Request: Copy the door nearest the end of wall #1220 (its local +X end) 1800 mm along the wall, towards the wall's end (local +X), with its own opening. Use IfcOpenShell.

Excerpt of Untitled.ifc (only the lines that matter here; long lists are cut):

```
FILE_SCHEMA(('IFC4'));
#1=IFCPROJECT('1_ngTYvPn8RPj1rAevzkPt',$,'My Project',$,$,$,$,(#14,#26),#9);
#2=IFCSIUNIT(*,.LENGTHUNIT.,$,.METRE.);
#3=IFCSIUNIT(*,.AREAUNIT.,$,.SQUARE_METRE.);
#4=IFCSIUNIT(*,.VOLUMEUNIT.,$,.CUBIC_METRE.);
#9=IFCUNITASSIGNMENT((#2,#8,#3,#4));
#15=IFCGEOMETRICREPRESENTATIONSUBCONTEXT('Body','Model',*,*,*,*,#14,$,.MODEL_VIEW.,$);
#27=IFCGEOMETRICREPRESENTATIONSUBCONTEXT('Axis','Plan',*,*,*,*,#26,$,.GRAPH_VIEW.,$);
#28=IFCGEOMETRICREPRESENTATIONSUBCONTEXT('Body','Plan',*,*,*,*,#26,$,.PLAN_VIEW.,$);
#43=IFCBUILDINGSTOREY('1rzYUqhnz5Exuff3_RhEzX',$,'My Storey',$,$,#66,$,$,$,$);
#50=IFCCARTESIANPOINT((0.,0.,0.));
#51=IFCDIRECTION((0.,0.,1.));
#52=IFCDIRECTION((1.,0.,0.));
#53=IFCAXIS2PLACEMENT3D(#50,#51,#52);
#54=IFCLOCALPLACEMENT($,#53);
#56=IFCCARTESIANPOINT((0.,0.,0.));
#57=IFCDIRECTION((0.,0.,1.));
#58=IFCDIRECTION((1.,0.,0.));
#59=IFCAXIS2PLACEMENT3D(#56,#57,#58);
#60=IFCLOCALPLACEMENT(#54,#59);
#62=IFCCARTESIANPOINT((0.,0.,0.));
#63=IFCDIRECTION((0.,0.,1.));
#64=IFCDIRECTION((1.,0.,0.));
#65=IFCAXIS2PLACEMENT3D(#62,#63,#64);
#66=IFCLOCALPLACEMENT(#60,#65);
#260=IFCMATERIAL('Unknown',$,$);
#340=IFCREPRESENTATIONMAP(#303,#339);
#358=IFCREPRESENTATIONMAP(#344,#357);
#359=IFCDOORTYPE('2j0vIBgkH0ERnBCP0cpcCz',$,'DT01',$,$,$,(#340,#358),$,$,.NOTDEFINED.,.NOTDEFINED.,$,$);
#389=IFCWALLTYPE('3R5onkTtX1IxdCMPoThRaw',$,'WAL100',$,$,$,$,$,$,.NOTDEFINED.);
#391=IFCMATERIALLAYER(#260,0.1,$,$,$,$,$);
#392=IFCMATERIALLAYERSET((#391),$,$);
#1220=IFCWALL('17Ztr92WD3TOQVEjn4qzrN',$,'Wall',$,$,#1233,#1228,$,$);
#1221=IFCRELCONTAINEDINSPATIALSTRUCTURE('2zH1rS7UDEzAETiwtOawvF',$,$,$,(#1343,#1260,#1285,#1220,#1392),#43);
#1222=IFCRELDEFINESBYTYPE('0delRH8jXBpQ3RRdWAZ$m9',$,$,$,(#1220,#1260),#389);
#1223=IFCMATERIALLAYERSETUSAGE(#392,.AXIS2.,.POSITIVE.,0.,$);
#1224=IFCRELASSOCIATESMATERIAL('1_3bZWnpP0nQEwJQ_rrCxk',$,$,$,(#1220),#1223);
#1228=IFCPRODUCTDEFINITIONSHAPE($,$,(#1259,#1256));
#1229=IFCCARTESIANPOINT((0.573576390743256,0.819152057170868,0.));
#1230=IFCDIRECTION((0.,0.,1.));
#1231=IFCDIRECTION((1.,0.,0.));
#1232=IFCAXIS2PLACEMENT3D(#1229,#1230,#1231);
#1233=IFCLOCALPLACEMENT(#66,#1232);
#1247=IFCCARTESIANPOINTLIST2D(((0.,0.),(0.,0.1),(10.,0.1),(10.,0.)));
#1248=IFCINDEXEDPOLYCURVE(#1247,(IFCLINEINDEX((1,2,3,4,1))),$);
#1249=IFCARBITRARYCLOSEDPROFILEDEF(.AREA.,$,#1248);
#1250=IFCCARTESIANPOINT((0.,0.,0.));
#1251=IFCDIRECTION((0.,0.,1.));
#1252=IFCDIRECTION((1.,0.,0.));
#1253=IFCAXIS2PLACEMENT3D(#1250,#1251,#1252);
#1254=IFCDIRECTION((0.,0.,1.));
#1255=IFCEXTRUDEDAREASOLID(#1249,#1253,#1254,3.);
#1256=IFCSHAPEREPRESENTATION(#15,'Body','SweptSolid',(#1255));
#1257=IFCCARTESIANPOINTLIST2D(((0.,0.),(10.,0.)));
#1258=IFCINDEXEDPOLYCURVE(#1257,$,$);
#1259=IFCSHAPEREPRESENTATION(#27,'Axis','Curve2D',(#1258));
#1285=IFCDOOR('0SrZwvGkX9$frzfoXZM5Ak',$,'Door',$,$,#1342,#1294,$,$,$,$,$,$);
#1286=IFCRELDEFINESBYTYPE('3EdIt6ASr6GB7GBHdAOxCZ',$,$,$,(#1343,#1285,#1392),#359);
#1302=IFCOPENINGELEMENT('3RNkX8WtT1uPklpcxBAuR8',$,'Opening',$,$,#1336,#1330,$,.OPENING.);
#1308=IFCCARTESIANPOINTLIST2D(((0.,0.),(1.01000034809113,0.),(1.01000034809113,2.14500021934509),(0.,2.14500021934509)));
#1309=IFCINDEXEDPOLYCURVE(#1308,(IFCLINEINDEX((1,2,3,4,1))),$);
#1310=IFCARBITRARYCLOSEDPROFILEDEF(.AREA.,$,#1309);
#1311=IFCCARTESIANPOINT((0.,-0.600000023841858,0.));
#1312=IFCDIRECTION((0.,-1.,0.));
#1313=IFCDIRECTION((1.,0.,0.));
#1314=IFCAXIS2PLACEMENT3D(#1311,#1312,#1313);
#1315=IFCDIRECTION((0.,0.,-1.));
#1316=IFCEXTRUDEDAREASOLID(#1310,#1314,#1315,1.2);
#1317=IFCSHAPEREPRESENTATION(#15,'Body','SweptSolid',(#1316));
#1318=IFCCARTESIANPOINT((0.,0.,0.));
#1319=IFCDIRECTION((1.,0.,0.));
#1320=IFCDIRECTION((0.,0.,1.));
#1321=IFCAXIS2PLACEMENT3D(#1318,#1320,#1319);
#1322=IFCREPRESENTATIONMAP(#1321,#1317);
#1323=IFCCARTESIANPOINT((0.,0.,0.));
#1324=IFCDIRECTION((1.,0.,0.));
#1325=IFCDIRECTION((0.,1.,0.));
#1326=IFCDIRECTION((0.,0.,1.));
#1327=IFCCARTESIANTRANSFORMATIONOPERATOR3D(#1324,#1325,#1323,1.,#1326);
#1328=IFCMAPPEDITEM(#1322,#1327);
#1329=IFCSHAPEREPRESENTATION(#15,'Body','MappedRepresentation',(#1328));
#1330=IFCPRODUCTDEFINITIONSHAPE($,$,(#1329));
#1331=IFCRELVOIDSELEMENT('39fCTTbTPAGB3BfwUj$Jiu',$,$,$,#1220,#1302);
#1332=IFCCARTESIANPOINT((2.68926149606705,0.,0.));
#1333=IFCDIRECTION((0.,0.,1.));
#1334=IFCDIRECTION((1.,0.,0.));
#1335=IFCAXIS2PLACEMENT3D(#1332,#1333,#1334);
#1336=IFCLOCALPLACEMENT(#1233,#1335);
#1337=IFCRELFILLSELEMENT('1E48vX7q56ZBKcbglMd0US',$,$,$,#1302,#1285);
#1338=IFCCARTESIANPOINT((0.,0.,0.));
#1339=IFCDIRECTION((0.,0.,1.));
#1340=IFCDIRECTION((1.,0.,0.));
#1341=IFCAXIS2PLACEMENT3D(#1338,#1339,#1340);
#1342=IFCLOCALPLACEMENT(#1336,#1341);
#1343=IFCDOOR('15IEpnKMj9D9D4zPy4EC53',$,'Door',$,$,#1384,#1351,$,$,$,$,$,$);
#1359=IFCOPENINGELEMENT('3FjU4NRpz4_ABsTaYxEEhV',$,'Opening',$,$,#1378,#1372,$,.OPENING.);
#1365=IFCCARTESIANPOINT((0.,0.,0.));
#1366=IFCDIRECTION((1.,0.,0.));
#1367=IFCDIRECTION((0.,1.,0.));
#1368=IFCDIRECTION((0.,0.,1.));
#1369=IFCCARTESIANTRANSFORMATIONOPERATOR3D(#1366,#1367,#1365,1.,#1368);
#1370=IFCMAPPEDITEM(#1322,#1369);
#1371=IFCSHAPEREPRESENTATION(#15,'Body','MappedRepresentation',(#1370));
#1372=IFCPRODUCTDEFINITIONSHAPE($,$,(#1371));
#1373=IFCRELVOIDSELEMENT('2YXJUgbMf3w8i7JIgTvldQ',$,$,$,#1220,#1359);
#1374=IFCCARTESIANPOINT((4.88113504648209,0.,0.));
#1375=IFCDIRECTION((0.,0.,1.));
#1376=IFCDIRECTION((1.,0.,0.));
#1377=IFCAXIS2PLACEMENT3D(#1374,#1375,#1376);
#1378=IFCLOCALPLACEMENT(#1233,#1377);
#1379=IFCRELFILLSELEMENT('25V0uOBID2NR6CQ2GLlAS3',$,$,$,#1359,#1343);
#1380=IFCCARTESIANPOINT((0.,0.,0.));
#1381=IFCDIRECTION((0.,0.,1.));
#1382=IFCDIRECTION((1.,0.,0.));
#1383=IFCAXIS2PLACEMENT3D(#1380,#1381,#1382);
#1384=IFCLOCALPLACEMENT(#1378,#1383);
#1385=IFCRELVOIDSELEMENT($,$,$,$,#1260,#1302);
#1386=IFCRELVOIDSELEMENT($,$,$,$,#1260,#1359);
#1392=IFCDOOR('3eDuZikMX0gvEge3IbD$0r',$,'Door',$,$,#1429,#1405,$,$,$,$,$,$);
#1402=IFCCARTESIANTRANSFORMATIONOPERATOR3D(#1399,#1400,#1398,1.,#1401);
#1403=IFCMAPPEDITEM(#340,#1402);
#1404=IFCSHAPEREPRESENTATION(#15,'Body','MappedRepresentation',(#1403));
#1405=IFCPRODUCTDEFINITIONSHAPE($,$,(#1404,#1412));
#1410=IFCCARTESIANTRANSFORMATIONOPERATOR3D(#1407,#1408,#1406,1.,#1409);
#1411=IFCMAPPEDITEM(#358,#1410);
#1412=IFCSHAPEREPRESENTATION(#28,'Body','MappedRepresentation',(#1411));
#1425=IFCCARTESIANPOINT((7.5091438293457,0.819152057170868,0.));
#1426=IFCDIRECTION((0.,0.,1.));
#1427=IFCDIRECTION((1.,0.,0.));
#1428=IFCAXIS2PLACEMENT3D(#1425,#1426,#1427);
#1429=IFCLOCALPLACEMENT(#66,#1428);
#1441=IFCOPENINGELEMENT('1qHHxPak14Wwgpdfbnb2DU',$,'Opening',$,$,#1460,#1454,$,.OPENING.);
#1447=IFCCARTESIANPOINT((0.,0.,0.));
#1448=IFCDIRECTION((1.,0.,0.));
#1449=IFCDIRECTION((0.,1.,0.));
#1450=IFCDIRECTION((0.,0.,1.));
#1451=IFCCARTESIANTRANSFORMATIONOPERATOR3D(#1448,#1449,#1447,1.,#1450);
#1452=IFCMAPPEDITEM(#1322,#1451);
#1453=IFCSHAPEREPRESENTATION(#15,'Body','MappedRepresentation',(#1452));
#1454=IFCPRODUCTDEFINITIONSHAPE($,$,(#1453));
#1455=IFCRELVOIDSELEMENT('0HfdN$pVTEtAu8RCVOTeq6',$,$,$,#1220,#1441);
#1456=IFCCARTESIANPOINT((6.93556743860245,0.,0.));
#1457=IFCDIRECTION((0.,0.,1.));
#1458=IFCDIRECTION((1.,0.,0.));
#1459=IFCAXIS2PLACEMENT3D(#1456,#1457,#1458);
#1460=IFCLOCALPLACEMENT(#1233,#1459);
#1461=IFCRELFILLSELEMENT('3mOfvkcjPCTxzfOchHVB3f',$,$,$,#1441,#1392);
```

```python
import ifcopenshell
import ifcopenshell.api.feature
import ifcopenshell.api.geometry
import ifcopenshell.api.root
import ifcopenshell.geom
import ifcopenshell.util.element
import ifcopenshell.util.placement
import ifcopenshell.util.shape

model = ifcopenshell.open("Untitled.ifc")
settings = ifcopenshell.geom.settings()


def volume(element):
    """Net volume in cubic metres, openings subtracted."""
    shape = ifcopenshell.geom.create_shape(settings, element)
    return ifcopenshell.util.shape.get_volume(shape.geometry)


door = model.by_guid("3eDuZikMX0gvEge3IbD$0r")
opening = door.FillsVoids[0].RelatingOpeningElement
wall = opening.VoidsElements[0].RelatingBuildingElement
before = volume(wall)
shift = ifcopenshell.util.placement.get_local_placement(wall.ObjectPlacement)[:3, 0] * 1.8

# copy_class copies the void relationship, type, container and properties, but no geometry.
new_opening = ifcopenshell.api.root.copy_class(model, product=opening)
new_opening.Representation = ifcopenshell.util.element.copy_deep(
    model, opening.Representation, exclude=["IfcGeometricRepresentationContext", "IfcRepresentationMap"]
)
new_door = ifcopenshell.api.root.copy_class(model, product=door)
new_door.Representation = ifcopenshell.util.element.copy_deep(
    model, door.Representation, exclude=["IfcGeometricRepresentationContext", "IfcRepresentationMap"]
)
ifcopenshell.api.feature.add_filling(model, opening=new_opening, element=new_door)

for old, new in ((opening, new_opening), (door, new_door)):
    matrix = ifcopenshell.util.placement.get_local_placement(old.ObjectPlacement)
    matrix[:3, 3] += shift
    ifcopenshell.api.geometry.edit_object_placement(model, product=new, matrix=matrix, is_si=False)

after = volume(wall)

print(f"wall volume {before:.3f} -> {after:.3f} m3")

model.write("Untitled_rev.ifc")
```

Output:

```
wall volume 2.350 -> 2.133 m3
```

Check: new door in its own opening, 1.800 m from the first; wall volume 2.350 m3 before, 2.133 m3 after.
